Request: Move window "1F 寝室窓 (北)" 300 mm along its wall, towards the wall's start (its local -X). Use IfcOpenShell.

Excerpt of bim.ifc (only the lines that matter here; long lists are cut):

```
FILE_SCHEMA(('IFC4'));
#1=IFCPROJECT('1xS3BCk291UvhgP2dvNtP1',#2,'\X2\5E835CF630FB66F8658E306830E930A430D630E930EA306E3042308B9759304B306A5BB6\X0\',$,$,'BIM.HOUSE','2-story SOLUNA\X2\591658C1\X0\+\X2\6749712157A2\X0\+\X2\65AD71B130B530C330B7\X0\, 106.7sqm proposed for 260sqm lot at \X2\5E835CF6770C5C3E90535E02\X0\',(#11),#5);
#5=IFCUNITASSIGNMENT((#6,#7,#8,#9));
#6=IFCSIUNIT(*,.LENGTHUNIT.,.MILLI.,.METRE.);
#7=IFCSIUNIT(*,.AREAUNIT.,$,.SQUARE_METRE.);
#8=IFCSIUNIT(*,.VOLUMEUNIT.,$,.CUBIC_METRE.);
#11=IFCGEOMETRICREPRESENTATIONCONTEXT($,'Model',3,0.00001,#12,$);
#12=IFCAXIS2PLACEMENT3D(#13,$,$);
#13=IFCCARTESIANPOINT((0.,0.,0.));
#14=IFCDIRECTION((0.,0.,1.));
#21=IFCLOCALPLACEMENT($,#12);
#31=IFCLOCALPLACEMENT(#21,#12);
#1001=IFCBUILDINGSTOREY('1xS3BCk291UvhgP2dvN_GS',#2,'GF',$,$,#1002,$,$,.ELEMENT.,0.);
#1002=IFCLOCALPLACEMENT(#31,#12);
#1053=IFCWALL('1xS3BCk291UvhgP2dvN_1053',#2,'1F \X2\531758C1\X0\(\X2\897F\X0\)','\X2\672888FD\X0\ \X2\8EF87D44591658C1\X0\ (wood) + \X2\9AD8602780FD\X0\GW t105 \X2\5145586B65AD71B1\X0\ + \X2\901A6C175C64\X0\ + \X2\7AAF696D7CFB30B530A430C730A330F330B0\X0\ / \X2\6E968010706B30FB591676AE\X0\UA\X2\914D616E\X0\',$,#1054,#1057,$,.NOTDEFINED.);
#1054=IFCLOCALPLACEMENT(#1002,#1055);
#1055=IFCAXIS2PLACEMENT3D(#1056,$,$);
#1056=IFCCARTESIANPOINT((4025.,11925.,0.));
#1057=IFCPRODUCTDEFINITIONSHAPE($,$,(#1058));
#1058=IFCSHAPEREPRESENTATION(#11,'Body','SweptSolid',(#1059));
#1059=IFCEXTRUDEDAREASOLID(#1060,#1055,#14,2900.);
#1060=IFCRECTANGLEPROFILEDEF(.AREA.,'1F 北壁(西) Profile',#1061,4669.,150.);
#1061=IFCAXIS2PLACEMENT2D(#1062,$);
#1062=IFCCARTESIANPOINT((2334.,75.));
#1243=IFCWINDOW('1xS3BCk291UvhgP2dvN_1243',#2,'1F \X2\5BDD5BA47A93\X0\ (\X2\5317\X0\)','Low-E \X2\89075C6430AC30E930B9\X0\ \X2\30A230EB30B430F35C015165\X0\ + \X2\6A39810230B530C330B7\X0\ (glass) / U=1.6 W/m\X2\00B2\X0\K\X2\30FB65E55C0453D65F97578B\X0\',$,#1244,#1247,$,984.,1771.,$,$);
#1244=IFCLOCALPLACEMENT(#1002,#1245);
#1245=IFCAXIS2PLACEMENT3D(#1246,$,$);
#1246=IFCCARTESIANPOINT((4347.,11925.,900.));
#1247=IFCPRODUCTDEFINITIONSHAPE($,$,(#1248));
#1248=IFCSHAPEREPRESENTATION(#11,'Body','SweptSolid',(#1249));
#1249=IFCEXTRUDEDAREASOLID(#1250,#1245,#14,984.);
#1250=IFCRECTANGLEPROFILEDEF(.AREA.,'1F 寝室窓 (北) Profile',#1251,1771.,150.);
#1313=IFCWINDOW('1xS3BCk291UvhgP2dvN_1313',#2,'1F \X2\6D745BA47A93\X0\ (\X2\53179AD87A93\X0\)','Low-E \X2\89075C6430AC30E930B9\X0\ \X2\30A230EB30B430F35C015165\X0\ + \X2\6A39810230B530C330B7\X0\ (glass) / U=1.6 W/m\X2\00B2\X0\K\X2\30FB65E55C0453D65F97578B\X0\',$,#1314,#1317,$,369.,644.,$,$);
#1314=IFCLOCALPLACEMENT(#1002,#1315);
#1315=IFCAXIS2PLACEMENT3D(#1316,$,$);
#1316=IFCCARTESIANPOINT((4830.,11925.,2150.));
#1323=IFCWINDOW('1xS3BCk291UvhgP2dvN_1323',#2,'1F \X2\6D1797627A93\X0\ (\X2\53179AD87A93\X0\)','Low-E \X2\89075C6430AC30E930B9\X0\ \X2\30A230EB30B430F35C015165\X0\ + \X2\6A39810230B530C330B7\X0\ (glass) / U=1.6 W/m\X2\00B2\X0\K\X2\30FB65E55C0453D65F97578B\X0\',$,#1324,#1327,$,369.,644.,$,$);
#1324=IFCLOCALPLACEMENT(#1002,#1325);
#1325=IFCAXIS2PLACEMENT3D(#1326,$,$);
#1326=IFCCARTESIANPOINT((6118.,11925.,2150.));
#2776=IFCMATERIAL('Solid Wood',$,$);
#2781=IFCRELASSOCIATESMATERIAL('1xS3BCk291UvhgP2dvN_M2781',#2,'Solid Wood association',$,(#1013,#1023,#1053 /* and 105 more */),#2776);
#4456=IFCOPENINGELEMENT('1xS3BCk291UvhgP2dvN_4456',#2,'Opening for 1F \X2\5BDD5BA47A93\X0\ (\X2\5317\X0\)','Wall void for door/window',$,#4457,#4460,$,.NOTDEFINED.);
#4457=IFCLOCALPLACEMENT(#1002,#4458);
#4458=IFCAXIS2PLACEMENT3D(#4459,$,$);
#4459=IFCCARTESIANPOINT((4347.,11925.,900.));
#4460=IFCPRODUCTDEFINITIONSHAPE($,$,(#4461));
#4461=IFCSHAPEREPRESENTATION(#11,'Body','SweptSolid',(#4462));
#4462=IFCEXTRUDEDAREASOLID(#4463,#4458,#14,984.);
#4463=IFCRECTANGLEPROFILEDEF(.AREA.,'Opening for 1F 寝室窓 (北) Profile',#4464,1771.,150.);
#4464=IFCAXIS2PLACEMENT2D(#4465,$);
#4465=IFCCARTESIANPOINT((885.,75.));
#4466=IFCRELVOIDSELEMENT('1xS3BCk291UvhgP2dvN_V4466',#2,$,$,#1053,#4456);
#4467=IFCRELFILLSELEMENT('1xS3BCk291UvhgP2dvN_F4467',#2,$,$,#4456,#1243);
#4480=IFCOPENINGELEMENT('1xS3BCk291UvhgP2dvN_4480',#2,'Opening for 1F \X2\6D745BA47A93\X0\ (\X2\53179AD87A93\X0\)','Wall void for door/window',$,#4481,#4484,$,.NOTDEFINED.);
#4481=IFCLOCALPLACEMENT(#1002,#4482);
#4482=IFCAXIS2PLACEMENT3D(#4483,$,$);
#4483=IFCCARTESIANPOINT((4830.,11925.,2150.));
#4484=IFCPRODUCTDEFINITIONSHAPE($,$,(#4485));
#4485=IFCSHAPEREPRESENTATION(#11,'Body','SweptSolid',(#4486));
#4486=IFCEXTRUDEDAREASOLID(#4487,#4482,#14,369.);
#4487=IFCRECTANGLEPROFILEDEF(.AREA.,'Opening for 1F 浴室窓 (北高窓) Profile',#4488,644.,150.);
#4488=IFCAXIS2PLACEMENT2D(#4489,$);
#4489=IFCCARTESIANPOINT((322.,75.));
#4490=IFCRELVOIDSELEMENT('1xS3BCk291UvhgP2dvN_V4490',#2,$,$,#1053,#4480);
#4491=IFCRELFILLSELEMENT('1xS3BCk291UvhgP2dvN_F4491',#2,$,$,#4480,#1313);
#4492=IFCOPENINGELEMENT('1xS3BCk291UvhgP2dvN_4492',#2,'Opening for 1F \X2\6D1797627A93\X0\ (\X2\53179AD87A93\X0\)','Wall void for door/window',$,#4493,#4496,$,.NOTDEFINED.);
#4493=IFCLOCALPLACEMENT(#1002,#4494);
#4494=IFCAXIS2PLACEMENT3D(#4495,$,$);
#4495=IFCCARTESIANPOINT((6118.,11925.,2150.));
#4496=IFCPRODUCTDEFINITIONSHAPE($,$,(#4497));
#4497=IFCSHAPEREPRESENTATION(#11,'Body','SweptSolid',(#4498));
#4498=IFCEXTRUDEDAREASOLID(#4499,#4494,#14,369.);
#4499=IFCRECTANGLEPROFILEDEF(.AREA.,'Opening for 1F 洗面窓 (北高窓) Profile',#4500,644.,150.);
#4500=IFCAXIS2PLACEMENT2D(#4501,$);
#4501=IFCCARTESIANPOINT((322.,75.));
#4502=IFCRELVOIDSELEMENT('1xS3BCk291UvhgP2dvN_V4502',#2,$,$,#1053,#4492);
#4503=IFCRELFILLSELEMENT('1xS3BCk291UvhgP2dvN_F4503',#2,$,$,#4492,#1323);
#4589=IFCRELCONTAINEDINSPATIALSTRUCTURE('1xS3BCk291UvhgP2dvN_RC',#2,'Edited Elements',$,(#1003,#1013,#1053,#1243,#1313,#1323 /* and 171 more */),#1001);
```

```python
import ifcopenshell
import ifcopenshell.api.geometry
import ifcopenshell.util.placement
import ifcopenshell.util.unit

model = ifcopenshell.open("bim.ifc")
unit_scale = ifcopenshell.util.unit.calculate_unit_scale(model)

window = model.by_guid("1xS3BCk291UvhgP2dvN_1243")
opening = window.FillsVoids[0].RelatingOpeningElement
wall = opening.VoidsElements[0].RelatingBuildingElement

wall_matrix = ifcopenshell.util.placement.get_local_placement(wall.ObjectPlacement)
shift = wall_matrix[:3, 0] * -0.3 / unit_scale
before = ifcopenshell.util.placement.get_local_placement(window.ObjectPlacement)[:3, 3].copy()

# The window is not placed relative to its opening, so move both.
for product in (opening, window):
    matrix = ifcopenshell.util.placement.get_local_placement(product.ObjectPlacement)
    matrix[:3, 3] += shift
    ifcopenshell.api.geometry.edit_object_placement(model, product=product, matrix=matrix, is_si=False)

after = ifcopenshell.util.placement.get_local_placement(window.ObjectPlacement)[:3, 3]
print("window moved by", (after - before).round(3) + 0.0)

model.write("bim-out.ifc")
```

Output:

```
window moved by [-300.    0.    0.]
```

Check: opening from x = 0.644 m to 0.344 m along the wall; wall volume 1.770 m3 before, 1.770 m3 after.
